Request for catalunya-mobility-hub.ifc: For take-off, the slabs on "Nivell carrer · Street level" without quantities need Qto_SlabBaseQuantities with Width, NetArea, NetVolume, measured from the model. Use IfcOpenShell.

First a look at what the model holds.

```python
import ifcopenshell
import ifcopenshell.util.element
import ifcopenshell.util.unit

model = ifcopenshell.open("catalunya-mobility-hub.ifc")
print(model.schema)
for unit_type in ("LENGTHUNIT", "AREAUNIT", "VOLUMEUNIT"):
    print(unit_type, ifcopenshell.util.unit.calculate_unit_scale(model, unit_type))
storey = next(s for s in model.by_type("IfcBuildingStorey") if s.Name == "Nivell carrer · Street level")
slabs = [e for e in ifcopenshell.util.element.get_decomposition(storey) if e.is_a("IfcSlab")]
for e in sorted(slabs, key=lambda e: e.id()):
    print(e.id(), e.is_a(), e.Name, list(ifcopenshell.util.element.get_psets(e, qtos_only=True)), sep=" | ")
```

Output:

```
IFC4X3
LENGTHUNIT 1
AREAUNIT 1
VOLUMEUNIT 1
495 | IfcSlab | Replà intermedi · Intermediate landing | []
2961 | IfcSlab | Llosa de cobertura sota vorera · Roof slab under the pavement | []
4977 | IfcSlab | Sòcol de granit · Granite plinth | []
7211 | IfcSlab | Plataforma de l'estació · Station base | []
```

```python
import ifcopenshell
import ifcopenshell.api.pset
import ifcopenshell.geom
import ifcopenshell.util.element
import ifcopenshell.util.shape
import ifcopenshell.util.unit

model = ifcopenshell.open("catalunya-mobility-hub.ifc")
unit_scale = ifcopenshell.util.unit.calculate_unit_scale(model)
area_scale = ifcopenshell.util.unit.calculate_unit_scale(model, "AREAUNIT")
volume_scale = ifcopenshell.util.unit.calculate_unit_scale(model, "VOLUMEUNIT")
settings = ifcopenshell.geom.settings()

storey = next(s for s in model.by_type("IfcBuildingStorey") if s.Name == "Nivell carrer · Street level")
slabs = [e for e in ifcopenshell.util.element.get_decomposition(storey) if e.is_a("IfcSlab")]

for e in sorted(slabs, key=lambda e: e.id()):
    if ifcopenshell.util.element.get_psets(e, qtos_only=True, should_inherit=False):
        continue
    # Geometry comes back in metres, in the element's own axes.
    shape = ifcopenshell.geom.create_shape(settings, e)
    values = {
        "Width": ifcopenshell.util.shape.get_z(shape.geometry) / unit_scale,
        "NetArea": ifcopenshell.util.shape.get_footprint_area(shape.geometry) / area_scale,
        "NetVolume": ifcopenshell.util.shape.get_volume(shape.geometry) / volume_scale,
    }
    qto = ifcopenshell.api.pset.add_qto(model, product=e, name="Qto_SlabBaseQuantities")
    ifcopenshell.api.pset.edit_qto(model, qto=qto, properties=values)
    print(e.id(), {k: round(v, 3) for k, v in values.items()})

model.write("catalunya-mobility-hub_v2.ifc")
```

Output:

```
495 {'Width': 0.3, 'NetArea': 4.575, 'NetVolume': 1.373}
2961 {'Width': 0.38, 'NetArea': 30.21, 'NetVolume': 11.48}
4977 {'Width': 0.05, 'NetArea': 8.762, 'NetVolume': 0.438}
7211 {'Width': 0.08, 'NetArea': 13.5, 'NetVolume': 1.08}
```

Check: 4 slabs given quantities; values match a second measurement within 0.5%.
